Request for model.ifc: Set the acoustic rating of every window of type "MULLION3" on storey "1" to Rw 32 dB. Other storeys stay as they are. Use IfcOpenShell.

First a look at what the model holds.

```python
import ifcopenshell
import ifcopenshell.util.element

model = ifcopenshell.open("model.ifc")
print(model.schema)
storey = next(s for s in model.by_type("IfcBuildingStorey") if s.Name == "1")
windows = [e for e in ifcopenshell.util.element.get_decomposition(storey) if e.is_a("IfcWindow")]
seen = {}
for e in windows:
    element_type = ifcopenshell.util.element.get_type(e)
    key = (element_type.Name if element_type != e and element_type else None, ifcopenshell.util.element.get_pset(e, "Pset_WindowCommon", "AcousticRating"))
    seen[key] = seen.get(key, 0) + 1
for (name, value), count in sorted(seen.items(), key=str):
    print(count, "x", name, "|", value)
```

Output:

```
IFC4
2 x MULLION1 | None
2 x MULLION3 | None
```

```python
import ifcopenshell
import ifcopenshell.api.pset
import ifcopenshell.util.element

model = ifcopenshell.open("model.ifc")

storey = next(s for s in model.by_type("IfcBuildingStorey") if s.Name == "1")
windows = [e for e in ifcopenshell.util.element.get_decomposition(storey) if e.is_a("IfcWindow")]

count = 0
for e in windows:
    element_type = ifcopenshell.util.element.get_type(e)
    if element_type in (None, e) or element_type.Name != "MULLION3":
        continue
    # add_pset returns the element's existing set when there is one.
    pset = ifcopenshell.api.pset.add_pset(model, product=e, name="Pset_WindowCommon")
    ifcopenshell.api.pset.edit_pset(model, pset=pset, properties={"AcousticRating": "Rw 32 dB"})
    count += 1

print(count, "windows updated")

model.write("model_rev.ifc")
```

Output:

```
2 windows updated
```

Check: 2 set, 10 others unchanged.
